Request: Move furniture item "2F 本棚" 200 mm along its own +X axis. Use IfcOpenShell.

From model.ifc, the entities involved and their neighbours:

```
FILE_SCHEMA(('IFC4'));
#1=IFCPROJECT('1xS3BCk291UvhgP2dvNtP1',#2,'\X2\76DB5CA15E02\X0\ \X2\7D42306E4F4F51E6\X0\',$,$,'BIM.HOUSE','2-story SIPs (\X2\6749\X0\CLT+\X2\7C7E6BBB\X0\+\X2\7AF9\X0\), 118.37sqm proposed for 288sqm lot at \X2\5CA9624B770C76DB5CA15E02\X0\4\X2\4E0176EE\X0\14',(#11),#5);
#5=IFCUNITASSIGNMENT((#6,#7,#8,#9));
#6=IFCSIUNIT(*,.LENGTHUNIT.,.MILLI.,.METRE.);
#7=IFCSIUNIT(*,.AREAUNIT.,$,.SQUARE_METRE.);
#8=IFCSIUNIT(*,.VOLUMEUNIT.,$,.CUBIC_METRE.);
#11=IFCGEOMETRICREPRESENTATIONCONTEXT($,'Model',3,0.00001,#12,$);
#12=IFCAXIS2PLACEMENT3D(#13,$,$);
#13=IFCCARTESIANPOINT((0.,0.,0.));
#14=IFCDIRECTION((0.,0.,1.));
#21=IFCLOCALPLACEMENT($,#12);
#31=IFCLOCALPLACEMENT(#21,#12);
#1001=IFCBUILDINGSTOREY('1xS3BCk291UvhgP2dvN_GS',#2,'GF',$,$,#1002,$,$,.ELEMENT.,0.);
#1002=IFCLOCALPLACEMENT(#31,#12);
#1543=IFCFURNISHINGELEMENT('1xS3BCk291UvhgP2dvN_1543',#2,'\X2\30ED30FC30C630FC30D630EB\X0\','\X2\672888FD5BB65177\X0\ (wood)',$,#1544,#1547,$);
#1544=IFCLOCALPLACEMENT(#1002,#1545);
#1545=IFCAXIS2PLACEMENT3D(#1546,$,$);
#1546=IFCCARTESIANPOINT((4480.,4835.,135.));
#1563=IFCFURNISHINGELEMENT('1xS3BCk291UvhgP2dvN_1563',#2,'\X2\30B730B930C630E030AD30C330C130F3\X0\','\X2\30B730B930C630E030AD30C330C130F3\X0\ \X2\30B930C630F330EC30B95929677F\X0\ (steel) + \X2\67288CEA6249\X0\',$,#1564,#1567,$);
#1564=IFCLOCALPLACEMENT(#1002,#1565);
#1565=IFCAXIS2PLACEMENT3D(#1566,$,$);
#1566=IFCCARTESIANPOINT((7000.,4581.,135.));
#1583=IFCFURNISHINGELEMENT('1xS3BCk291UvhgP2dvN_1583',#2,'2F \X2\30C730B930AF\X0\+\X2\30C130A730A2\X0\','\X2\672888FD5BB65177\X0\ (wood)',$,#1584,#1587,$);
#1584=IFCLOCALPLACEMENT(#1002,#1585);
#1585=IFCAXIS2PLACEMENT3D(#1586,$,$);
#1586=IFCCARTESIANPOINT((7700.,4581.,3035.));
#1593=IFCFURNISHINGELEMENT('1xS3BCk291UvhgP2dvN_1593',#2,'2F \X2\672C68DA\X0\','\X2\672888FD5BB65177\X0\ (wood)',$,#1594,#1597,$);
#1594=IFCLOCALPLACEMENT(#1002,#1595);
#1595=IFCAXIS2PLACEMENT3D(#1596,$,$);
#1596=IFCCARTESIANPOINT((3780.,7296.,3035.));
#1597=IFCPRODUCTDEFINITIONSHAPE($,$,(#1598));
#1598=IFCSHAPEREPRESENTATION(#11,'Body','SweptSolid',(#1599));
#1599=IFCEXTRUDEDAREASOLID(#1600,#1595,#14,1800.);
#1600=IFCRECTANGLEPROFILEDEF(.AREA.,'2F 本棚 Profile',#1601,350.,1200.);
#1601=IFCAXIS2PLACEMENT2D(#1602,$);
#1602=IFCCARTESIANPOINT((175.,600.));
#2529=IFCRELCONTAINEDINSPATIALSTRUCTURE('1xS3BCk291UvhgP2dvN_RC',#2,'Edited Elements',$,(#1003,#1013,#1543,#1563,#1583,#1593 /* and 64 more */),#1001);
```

```python
import ifcopenshell
import ifcopenshell.api.geometry
import ifcopenshell.util.placement
import ifcopenshell.util.unit

model = ifcopenshell.open("model.ifc")
unit_scale = ifcopenshell.util.unit.calculate_unit_scale(model)

item = model.by_guid("1xS3BCk291UvhgP2dvN_1593")
matrix = ifcopenshell.util.placement.get_local_placement(item.ObjectPlacement)
matrix[:3, 3] += matrix[:3, 0] * 0.2 / unit_scale
ifcopenshell.api.geometry.edit_object_placement(model, product=item, matrix=matrix, is_si=False)

print(ifcopenshell.util.placement.get_local_placement(item.ObjectPlacement).round(3) + 0.0)

model.write("model_updated.ifc")
```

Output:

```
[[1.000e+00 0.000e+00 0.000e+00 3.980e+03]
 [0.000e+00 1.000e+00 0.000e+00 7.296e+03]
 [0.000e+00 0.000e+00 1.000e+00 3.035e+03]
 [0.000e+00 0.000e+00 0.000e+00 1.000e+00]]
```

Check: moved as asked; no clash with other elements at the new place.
